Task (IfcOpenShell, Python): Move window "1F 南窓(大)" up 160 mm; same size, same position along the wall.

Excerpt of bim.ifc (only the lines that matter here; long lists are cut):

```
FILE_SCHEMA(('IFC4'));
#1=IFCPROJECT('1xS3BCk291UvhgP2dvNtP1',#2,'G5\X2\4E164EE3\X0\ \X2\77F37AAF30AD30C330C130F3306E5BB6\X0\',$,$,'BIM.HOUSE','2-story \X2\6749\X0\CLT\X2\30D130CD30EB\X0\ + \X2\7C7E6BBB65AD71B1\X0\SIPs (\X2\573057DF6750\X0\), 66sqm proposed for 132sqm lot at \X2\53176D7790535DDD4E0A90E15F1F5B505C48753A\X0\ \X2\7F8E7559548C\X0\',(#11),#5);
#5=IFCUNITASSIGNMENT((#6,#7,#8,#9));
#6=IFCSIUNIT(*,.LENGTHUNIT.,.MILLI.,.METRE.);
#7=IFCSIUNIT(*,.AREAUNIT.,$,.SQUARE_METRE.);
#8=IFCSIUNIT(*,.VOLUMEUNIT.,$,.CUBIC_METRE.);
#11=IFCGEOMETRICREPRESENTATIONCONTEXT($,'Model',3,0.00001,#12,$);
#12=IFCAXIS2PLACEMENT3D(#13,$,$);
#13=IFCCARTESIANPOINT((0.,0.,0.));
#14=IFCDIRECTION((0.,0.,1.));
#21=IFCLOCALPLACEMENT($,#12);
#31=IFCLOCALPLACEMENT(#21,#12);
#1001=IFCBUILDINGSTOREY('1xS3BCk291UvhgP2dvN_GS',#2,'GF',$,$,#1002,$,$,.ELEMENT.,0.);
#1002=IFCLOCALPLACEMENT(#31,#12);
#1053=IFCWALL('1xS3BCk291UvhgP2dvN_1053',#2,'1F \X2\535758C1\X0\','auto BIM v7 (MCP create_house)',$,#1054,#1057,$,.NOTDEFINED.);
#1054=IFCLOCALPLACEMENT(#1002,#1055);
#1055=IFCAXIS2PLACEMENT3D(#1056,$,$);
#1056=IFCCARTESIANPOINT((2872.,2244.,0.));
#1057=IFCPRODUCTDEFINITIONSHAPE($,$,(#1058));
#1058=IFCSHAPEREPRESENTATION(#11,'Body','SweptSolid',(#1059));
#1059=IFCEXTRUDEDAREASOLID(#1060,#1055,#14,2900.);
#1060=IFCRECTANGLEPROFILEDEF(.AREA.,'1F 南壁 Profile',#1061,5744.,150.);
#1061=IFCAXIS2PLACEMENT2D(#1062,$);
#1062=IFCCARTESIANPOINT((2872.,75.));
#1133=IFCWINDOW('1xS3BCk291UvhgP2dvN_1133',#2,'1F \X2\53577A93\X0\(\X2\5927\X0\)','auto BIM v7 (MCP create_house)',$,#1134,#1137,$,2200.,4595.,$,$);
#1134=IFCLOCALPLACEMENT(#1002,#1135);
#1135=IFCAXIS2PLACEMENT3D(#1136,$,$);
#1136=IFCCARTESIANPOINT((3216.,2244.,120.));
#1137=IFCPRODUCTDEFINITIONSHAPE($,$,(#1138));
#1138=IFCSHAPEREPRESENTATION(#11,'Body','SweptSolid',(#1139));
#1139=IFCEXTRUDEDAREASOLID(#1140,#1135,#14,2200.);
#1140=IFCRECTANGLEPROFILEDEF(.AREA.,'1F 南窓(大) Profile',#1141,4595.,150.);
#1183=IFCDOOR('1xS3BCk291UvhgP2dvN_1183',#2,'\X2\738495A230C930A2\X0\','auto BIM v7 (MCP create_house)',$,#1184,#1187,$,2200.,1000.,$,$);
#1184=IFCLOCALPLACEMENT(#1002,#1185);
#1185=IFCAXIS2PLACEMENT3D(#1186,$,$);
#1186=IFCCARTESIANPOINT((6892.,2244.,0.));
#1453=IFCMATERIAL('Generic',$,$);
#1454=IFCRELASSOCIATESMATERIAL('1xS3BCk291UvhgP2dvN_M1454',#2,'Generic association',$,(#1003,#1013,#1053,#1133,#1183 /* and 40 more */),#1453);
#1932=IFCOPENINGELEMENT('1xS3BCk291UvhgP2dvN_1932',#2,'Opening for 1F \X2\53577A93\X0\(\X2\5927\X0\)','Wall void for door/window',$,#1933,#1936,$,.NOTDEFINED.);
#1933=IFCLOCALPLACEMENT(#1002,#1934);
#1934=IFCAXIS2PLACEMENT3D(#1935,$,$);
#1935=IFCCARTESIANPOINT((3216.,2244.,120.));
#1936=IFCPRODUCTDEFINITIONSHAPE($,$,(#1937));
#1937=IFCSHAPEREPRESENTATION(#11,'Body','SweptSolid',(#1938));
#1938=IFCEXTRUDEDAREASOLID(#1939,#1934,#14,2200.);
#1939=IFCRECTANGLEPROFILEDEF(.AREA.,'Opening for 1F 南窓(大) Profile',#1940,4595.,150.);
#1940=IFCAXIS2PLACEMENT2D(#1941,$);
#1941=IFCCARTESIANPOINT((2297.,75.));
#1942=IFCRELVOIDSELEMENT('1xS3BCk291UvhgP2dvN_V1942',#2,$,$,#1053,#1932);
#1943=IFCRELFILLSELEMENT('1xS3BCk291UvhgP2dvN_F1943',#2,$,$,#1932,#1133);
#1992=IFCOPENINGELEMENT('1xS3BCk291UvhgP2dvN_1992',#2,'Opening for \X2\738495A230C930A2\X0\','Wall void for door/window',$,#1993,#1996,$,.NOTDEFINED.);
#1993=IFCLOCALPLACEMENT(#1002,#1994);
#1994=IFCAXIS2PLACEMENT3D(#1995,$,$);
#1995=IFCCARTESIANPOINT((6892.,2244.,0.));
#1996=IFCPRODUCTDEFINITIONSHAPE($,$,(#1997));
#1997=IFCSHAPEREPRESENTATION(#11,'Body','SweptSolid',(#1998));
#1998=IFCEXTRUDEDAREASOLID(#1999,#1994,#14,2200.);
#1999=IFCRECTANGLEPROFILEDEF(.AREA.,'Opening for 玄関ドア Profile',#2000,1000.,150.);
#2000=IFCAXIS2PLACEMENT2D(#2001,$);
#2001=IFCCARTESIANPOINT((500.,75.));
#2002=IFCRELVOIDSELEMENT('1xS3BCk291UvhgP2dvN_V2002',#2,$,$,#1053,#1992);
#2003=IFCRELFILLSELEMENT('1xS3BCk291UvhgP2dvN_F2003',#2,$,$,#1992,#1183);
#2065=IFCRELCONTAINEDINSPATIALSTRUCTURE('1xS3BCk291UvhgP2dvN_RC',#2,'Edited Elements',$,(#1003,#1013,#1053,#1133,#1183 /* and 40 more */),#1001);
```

```python
import numpy as np
import ifcopenshell
import ifcopenshell.api.geometry
import ifcopenshell.util.placement
import ifcopenshell.util.unit

model = ifcopenshell.open("bim.ifc")
unit_scale = ifcopenshell.util.unit.calculate_unit_scale(model)

window = model.by_guid("1xS3BCk291UvhgP2dvN_1133")
opening = window.FillsVoids[0].RelatingOpeningElement
dz = 0.16 / unit_scale

shift = np.array([0.0, 0.0, dz])
# The window is not placed relative to its opening, so move both.
for product in (opening, window):
    matrix = ifcopenshell.util.placement.get_local_placement(product.ObjectPlacement)
    matrix[:3, 3] += shift
    ifcopenshell.api.geometry.edit_object_placement(model, product=product, matrix=matrix, is_si=False)

print(f"moved by {dz * unit_scale:+.3f} m")

model.write("bim_rev.ifc")
```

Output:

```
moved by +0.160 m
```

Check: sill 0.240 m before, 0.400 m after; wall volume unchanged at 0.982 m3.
